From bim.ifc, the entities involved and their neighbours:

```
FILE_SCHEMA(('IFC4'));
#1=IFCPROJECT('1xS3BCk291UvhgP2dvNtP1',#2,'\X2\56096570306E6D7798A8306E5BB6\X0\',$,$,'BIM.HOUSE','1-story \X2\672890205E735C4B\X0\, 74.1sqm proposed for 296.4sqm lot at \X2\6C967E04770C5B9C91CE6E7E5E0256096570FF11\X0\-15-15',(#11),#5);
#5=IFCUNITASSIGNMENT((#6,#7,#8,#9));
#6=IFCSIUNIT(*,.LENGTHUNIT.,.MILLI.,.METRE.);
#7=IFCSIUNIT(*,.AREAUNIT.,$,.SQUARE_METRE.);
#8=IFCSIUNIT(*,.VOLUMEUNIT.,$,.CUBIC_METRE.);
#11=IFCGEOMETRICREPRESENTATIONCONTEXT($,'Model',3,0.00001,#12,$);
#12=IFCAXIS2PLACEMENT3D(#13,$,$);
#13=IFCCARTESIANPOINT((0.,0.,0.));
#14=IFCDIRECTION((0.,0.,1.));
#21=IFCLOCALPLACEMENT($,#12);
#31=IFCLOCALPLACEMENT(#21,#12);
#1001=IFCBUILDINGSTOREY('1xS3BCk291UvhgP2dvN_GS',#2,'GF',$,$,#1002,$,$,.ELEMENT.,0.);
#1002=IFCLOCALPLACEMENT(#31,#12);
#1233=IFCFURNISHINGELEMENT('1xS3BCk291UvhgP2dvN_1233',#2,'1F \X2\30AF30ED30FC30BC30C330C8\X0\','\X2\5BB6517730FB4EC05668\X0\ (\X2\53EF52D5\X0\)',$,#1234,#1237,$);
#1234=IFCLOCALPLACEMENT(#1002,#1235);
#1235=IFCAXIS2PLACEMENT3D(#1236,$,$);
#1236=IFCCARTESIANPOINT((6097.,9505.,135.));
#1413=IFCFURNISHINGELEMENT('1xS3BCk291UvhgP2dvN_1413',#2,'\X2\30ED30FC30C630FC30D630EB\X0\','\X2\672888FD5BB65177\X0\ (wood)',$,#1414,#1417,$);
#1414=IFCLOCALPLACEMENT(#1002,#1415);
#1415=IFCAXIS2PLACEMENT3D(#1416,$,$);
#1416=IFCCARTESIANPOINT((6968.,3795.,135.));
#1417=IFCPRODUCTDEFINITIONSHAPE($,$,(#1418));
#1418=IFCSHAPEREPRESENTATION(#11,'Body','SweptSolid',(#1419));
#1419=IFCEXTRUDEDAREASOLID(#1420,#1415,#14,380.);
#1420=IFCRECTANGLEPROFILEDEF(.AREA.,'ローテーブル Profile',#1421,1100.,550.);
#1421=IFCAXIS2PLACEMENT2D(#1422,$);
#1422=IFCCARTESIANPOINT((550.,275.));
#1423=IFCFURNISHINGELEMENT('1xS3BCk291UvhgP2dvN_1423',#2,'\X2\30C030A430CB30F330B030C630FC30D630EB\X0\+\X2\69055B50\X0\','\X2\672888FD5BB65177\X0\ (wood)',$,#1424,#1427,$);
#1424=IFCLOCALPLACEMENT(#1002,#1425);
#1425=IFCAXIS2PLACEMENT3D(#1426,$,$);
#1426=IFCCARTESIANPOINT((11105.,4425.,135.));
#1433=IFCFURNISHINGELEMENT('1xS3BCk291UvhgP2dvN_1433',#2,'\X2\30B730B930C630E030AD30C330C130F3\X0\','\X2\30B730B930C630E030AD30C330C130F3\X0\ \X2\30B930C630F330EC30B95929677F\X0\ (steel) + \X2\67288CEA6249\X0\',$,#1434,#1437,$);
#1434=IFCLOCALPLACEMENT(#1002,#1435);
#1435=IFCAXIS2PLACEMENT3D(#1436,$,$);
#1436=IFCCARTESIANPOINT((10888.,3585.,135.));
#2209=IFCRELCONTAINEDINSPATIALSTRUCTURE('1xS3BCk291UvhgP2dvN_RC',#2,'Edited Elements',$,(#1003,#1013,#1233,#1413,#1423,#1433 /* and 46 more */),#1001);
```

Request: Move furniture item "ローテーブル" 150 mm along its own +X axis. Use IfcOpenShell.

```python
import ifcopenshell
import ifcopenshell.api.geometry
import ifcopenshell.util.placement
import ifcopenshell.util.unit

model = ifcopenshell.open("bim.ifc")
unit_scale = ifcopenshell.util.unit.calculate_unit_scale(model)

item = model.by_id(1413)
matrix = ifcopenshell.util.placement.get_local_placement(item.ObjectPlacement)
matrix[:3, 3] += matrix[:3, 0] * 0.15 / unit_scale
ifcopenshell.api.geometry.edit_object_placement(model, product=item, matrix=matrix, is_si=False)

print(ifcopenshell.util.placement.get_local_placement(item.ObjectPlacement).round(3) + 0.0)

model.write("bim_rev.ifc")
```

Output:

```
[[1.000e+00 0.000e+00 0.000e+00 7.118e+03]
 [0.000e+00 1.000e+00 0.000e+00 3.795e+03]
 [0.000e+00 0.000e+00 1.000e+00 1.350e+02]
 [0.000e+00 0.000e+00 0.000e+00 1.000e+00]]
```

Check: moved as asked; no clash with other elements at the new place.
